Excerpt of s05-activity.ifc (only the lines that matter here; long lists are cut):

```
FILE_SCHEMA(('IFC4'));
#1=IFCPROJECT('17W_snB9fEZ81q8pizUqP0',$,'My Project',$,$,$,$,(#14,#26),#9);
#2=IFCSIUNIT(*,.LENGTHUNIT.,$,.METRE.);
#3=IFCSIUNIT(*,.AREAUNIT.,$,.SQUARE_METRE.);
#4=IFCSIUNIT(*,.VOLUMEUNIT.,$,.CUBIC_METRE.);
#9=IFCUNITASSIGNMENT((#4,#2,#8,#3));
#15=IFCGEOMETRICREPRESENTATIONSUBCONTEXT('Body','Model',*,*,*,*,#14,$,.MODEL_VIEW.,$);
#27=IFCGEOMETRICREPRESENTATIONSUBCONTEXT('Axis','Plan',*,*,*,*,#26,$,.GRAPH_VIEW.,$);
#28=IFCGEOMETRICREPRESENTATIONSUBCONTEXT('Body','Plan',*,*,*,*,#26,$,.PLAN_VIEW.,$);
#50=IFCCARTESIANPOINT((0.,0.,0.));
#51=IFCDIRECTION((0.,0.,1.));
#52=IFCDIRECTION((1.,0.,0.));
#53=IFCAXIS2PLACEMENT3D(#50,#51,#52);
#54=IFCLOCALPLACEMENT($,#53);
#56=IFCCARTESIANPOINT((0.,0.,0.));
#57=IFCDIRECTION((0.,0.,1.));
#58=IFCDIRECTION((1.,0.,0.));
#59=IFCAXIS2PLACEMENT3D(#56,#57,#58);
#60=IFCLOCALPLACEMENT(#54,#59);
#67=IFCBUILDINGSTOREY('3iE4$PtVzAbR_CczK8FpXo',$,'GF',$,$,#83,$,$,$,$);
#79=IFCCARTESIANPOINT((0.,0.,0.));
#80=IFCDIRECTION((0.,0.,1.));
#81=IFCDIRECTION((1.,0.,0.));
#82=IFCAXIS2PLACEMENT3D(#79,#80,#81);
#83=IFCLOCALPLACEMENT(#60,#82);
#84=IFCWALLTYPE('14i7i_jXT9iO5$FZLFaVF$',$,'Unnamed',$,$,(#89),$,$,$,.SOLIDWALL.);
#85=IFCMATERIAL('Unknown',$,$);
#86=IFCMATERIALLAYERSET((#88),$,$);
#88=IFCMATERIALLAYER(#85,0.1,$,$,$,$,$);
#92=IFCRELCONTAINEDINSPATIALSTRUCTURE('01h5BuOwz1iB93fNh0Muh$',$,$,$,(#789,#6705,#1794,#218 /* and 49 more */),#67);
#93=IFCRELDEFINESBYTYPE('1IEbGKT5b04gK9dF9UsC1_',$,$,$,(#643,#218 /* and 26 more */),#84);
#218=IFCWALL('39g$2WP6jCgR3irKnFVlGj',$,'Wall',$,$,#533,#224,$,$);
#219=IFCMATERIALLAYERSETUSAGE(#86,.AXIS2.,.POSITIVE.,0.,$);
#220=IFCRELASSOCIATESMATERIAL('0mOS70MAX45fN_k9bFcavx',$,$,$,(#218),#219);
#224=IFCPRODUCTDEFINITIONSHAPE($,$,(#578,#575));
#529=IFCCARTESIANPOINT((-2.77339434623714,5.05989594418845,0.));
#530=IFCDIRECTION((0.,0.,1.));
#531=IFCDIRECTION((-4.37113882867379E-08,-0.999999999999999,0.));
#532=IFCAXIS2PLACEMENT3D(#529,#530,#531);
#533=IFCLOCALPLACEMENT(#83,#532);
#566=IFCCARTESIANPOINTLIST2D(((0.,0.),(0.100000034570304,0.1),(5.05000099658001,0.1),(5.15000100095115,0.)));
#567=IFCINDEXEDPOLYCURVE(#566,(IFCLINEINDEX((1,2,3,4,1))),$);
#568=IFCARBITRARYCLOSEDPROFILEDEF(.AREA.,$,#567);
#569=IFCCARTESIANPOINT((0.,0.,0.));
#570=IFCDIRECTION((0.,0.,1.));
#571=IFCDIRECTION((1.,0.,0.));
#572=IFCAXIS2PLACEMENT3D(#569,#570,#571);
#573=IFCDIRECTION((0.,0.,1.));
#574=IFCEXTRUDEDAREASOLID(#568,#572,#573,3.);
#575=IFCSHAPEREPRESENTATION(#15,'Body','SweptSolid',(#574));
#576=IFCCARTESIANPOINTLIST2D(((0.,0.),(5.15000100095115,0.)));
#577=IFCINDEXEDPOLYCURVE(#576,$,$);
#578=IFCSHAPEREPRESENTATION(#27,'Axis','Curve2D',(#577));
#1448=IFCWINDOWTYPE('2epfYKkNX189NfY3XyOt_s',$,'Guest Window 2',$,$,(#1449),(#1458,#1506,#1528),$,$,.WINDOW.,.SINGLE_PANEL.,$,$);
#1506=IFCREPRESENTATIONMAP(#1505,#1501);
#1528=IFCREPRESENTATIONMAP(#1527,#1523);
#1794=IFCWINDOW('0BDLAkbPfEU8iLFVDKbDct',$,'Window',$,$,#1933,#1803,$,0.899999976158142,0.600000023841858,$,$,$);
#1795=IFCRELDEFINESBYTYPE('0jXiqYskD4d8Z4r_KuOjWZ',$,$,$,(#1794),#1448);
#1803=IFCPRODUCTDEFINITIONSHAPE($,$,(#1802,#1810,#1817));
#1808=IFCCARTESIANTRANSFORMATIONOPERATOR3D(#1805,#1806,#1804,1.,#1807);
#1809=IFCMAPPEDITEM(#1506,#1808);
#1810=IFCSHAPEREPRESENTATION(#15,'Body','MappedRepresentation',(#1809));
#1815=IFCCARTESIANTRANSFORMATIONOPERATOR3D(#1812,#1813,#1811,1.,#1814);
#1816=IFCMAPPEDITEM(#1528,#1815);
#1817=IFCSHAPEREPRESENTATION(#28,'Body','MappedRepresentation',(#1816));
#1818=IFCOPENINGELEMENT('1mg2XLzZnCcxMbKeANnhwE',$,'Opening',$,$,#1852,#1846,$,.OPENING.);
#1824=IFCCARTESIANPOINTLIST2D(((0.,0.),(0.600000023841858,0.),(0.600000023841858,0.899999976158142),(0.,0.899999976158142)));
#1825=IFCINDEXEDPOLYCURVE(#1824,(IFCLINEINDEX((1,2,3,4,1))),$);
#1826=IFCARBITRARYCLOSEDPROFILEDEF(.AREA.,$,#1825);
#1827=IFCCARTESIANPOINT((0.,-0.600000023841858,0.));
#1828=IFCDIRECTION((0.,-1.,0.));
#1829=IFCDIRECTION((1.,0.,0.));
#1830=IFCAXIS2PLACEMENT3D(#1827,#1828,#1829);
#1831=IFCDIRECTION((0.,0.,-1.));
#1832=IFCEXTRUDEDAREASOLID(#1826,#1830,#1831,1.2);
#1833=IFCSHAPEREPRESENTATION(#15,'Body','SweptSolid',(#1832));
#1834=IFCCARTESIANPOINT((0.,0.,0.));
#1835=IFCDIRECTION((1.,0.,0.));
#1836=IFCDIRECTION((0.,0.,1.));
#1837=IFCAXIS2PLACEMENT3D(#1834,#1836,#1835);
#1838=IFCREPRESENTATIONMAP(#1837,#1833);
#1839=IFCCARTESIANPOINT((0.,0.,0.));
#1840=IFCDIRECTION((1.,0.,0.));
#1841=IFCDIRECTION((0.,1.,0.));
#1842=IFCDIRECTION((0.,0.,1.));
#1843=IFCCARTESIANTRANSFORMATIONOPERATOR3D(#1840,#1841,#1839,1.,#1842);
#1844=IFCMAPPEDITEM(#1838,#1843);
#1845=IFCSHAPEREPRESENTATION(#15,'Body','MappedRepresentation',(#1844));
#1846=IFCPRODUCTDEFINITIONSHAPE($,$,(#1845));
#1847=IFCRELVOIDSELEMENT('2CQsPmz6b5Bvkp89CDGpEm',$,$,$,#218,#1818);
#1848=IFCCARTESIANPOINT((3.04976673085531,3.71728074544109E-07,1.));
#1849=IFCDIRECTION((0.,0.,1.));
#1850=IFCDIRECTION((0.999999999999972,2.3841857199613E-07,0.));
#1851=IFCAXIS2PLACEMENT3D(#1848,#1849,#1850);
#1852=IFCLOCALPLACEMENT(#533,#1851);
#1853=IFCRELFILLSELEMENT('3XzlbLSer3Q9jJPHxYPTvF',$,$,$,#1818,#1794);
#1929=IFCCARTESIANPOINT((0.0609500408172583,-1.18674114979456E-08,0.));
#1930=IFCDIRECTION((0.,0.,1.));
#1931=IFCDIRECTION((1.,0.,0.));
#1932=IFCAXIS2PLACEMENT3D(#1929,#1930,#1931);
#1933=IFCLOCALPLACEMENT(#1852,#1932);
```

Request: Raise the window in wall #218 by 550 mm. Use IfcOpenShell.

```python
import numpy as np
import ifcopenshell
import ifcopenshell.api.geometry
import ifcopenshell.util.placement
import ifcopenshell.util.unit

model = ifcopenshell.open("s05-activity.ifc")
unit_scale = ifcopenshell.util.unit.calculate_unit_scale(model)

window = model.by_id(1794)
opening = window.FillsVoids[0].RelatingOpeningElement
dz = 0.55 / unit_scale

shift = np.array([0.0, 0.0, dz])
# The window is placed relative to its opening, so it follows when the opening moves.
matrix = ifcopenshell.util.placement.get_local_placement(opening.ObjectPlacement)
matrix[:3, 3] += shift
ifcopenshell.api.geometry.edit_object_placement(
    model, product=opening, matrix=matrix, is_si=False, should_transform_children=True
)

print(f"moved by {dz * unit_scale:+.3f} m")

model.write("s05-activity_rev.ifc")
```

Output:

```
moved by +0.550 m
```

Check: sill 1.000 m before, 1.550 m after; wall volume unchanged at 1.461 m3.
